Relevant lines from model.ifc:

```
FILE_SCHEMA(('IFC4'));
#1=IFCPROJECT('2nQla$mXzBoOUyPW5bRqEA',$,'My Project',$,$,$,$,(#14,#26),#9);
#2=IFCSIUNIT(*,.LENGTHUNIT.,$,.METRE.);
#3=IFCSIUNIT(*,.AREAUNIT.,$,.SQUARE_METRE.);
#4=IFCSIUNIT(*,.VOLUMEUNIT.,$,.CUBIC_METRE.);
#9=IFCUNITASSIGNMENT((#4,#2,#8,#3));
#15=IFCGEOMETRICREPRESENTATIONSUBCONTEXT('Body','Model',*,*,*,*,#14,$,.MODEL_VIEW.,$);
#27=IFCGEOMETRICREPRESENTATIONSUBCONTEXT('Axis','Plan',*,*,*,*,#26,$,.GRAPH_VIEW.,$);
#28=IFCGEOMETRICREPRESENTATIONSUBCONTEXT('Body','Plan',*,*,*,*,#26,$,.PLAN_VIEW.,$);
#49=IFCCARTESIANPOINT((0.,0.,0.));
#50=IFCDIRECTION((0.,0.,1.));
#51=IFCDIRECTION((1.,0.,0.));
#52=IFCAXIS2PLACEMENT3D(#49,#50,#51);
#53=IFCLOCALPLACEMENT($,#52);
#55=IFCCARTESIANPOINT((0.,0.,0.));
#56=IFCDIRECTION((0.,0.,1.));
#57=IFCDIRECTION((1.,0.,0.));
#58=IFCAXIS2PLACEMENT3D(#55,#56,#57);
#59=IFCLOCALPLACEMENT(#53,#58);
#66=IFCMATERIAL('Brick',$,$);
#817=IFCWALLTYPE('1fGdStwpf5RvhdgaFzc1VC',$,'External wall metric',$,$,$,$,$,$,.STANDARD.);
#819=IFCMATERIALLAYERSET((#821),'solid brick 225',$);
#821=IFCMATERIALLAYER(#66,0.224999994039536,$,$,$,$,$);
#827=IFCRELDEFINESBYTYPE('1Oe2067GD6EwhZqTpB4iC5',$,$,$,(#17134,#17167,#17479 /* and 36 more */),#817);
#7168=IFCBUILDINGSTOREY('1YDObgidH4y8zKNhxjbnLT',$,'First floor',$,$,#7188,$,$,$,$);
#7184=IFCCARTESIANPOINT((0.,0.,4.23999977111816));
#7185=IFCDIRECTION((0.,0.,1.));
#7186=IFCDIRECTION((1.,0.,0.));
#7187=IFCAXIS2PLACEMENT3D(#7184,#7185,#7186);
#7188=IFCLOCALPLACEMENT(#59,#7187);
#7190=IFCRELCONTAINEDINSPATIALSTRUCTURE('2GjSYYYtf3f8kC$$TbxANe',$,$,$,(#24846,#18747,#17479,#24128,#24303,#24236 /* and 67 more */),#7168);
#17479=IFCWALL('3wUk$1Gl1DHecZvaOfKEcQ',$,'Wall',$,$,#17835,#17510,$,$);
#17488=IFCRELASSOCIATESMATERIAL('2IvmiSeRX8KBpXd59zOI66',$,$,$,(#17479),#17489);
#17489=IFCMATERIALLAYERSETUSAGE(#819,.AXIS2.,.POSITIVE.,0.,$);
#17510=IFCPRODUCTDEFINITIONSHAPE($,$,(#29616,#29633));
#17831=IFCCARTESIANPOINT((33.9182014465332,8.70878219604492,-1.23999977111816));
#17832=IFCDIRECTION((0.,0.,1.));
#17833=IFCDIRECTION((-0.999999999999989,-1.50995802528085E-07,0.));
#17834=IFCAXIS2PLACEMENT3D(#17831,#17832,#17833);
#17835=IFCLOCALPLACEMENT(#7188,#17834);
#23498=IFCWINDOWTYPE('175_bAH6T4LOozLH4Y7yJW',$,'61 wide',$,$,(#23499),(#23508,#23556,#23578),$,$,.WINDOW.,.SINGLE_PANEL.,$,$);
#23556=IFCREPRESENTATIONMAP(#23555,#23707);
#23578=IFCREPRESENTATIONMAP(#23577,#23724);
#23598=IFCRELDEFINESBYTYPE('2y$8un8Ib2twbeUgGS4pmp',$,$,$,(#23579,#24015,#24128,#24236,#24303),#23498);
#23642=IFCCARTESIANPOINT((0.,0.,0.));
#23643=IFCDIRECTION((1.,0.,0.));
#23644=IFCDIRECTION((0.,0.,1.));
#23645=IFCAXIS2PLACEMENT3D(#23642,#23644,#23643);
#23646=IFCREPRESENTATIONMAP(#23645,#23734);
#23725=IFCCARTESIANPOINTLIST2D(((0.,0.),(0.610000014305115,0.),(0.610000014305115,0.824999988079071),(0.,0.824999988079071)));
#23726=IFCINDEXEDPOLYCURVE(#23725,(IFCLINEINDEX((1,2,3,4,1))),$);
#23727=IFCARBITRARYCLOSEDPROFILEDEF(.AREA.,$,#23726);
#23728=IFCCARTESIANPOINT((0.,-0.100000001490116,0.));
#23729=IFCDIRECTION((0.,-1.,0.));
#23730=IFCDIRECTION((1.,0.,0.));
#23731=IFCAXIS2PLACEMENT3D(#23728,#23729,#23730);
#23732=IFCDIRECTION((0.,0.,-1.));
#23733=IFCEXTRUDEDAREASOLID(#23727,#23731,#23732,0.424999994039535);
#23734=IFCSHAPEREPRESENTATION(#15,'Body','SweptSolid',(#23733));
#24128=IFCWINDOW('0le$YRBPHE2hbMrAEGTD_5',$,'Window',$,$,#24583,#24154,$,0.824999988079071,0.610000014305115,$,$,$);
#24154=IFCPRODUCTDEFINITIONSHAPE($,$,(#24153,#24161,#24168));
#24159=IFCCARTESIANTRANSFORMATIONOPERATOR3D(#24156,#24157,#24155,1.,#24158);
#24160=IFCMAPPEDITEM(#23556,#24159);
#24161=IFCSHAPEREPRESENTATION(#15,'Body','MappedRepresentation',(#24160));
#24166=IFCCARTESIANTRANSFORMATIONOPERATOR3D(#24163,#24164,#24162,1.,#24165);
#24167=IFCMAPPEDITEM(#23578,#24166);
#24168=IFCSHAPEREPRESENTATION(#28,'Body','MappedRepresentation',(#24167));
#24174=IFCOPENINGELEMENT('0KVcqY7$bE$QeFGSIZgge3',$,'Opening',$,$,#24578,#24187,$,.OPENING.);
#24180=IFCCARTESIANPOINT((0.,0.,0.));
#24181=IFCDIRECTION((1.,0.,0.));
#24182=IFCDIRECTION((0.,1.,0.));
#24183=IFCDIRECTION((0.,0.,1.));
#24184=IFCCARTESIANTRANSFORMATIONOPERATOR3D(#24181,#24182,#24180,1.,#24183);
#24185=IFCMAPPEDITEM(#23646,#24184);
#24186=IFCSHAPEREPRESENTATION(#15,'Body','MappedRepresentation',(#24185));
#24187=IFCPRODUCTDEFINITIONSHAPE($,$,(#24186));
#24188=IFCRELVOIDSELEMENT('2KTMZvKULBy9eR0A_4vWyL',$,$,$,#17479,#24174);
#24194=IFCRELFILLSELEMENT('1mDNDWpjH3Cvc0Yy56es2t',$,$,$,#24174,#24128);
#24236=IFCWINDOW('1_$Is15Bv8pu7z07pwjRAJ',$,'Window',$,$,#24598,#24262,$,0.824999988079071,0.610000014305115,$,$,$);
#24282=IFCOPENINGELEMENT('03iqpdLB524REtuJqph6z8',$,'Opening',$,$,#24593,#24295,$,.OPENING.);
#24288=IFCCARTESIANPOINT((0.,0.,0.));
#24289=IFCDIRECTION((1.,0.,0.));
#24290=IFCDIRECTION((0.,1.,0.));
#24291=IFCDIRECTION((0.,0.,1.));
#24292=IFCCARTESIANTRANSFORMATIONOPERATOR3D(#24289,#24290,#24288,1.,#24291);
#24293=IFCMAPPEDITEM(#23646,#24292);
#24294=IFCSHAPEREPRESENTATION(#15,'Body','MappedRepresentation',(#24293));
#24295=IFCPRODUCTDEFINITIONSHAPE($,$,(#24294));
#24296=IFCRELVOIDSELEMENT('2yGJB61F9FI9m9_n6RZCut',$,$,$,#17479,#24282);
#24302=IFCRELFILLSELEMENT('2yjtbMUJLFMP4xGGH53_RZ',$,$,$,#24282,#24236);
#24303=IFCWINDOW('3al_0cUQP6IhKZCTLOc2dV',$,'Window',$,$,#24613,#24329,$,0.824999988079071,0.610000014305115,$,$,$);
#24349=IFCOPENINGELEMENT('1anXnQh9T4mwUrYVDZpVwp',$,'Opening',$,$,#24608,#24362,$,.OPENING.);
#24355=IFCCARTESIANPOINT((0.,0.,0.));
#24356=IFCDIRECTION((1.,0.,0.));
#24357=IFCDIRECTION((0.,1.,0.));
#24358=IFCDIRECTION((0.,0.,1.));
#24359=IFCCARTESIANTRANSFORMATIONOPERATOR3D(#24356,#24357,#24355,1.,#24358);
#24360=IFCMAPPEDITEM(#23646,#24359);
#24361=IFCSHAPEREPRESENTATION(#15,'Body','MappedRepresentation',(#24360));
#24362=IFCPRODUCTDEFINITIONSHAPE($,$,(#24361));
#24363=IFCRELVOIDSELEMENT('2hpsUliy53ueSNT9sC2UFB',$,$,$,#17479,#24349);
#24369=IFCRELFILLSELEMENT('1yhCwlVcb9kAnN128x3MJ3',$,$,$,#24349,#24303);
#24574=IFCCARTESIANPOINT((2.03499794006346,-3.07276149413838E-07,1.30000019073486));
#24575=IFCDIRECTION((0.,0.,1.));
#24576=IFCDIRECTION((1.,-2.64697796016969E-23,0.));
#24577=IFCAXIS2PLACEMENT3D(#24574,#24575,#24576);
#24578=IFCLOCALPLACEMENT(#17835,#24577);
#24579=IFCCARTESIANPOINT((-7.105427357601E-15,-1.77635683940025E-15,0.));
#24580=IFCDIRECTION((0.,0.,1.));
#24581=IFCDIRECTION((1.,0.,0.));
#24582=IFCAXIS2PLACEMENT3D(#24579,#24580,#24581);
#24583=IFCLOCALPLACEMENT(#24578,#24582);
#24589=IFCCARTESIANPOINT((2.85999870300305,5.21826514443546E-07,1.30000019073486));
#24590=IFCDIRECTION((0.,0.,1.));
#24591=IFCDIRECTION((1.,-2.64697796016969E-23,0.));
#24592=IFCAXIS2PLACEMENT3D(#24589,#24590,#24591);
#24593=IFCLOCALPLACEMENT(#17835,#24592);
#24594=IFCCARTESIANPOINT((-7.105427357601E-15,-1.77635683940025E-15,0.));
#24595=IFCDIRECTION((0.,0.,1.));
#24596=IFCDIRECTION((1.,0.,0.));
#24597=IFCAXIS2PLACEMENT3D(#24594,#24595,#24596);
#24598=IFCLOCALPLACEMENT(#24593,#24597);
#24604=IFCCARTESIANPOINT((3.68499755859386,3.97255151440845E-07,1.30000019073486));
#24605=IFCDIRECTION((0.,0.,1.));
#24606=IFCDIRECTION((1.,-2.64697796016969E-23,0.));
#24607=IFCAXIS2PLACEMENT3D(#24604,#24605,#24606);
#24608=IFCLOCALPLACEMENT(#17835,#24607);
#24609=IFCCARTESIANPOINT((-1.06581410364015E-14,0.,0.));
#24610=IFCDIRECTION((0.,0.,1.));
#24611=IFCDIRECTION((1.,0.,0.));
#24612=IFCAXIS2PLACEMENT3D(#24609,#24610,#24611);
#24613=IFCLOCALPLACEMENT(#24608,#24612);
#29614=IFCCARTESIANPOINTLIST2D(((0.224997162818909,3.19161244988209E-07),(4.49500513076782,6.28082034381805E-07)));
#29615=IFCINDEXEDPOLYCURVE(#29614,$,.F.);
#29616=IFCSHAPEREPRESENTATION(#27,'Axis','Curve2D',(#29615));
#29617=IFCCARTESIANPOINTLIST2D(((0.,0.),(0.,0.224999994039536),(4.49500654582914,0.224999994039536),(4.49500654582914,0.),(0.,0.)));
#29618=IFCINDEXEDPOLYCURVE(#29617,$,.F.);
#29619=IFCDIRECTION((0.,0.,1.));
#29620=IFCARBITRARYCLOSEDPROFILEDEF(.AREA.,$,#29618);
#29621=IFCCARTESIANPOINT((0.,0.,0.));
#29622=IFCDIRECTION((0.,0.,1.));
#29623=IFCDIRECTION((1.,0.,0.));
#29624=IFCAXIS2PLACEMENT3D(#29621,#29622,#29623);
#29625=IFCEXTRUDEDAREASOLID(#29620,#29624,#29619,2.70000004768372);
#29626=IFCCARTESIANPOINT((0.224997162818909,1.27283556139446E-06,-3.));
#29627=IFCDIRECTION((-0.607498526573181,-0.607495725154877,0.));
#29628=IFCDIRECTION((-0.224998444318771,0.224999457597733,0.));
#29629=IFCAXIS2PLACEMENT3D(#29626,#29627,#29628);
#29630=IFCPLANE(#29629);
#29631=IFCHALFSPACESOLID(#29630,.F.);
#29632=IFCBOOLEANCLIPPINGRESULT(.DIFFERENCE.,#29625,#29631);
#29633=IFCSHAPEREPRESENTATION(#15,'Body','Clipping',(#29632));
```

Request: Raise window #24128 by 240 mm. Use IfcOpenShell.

```python
import numpy as np
import ifcopenshell
import ifcopenshell.api.geometry
import ifcopenshell.util.placement
import ifcopenshell.util.unit

model = ifcopenshell.open("model.ifc")
unit_scale = ifcopenshell.util.unit.calculate_unit_scale(model)

window = model.by_guid("0le$YRBPHE2hbMrAEGTD_5")
opening = window.FillsVoids[0].RelatingOpeningElement
dz = 0.24 / unit_scale

shift = np.array([0.0, 0.0, dz])
# The window is placed relative to its opening, so it follows when the opening moves.
matrix = ifcopenshell.util.placement.get_local_placement(opening.ObjectPlacement)
matrix[:3, 3] += shift
ifcopenshell.api.geometry.edit_object_placement(
    model, product=opening, matrix=matrix, is_si=False, should_transform_children=True
)

print(f"moved by {dz * unit_scale:+.3f} m")

model.write("model_v2.ifc")
```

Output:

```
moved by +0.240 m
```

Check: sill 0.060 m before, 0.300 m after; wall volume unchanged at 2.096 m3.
